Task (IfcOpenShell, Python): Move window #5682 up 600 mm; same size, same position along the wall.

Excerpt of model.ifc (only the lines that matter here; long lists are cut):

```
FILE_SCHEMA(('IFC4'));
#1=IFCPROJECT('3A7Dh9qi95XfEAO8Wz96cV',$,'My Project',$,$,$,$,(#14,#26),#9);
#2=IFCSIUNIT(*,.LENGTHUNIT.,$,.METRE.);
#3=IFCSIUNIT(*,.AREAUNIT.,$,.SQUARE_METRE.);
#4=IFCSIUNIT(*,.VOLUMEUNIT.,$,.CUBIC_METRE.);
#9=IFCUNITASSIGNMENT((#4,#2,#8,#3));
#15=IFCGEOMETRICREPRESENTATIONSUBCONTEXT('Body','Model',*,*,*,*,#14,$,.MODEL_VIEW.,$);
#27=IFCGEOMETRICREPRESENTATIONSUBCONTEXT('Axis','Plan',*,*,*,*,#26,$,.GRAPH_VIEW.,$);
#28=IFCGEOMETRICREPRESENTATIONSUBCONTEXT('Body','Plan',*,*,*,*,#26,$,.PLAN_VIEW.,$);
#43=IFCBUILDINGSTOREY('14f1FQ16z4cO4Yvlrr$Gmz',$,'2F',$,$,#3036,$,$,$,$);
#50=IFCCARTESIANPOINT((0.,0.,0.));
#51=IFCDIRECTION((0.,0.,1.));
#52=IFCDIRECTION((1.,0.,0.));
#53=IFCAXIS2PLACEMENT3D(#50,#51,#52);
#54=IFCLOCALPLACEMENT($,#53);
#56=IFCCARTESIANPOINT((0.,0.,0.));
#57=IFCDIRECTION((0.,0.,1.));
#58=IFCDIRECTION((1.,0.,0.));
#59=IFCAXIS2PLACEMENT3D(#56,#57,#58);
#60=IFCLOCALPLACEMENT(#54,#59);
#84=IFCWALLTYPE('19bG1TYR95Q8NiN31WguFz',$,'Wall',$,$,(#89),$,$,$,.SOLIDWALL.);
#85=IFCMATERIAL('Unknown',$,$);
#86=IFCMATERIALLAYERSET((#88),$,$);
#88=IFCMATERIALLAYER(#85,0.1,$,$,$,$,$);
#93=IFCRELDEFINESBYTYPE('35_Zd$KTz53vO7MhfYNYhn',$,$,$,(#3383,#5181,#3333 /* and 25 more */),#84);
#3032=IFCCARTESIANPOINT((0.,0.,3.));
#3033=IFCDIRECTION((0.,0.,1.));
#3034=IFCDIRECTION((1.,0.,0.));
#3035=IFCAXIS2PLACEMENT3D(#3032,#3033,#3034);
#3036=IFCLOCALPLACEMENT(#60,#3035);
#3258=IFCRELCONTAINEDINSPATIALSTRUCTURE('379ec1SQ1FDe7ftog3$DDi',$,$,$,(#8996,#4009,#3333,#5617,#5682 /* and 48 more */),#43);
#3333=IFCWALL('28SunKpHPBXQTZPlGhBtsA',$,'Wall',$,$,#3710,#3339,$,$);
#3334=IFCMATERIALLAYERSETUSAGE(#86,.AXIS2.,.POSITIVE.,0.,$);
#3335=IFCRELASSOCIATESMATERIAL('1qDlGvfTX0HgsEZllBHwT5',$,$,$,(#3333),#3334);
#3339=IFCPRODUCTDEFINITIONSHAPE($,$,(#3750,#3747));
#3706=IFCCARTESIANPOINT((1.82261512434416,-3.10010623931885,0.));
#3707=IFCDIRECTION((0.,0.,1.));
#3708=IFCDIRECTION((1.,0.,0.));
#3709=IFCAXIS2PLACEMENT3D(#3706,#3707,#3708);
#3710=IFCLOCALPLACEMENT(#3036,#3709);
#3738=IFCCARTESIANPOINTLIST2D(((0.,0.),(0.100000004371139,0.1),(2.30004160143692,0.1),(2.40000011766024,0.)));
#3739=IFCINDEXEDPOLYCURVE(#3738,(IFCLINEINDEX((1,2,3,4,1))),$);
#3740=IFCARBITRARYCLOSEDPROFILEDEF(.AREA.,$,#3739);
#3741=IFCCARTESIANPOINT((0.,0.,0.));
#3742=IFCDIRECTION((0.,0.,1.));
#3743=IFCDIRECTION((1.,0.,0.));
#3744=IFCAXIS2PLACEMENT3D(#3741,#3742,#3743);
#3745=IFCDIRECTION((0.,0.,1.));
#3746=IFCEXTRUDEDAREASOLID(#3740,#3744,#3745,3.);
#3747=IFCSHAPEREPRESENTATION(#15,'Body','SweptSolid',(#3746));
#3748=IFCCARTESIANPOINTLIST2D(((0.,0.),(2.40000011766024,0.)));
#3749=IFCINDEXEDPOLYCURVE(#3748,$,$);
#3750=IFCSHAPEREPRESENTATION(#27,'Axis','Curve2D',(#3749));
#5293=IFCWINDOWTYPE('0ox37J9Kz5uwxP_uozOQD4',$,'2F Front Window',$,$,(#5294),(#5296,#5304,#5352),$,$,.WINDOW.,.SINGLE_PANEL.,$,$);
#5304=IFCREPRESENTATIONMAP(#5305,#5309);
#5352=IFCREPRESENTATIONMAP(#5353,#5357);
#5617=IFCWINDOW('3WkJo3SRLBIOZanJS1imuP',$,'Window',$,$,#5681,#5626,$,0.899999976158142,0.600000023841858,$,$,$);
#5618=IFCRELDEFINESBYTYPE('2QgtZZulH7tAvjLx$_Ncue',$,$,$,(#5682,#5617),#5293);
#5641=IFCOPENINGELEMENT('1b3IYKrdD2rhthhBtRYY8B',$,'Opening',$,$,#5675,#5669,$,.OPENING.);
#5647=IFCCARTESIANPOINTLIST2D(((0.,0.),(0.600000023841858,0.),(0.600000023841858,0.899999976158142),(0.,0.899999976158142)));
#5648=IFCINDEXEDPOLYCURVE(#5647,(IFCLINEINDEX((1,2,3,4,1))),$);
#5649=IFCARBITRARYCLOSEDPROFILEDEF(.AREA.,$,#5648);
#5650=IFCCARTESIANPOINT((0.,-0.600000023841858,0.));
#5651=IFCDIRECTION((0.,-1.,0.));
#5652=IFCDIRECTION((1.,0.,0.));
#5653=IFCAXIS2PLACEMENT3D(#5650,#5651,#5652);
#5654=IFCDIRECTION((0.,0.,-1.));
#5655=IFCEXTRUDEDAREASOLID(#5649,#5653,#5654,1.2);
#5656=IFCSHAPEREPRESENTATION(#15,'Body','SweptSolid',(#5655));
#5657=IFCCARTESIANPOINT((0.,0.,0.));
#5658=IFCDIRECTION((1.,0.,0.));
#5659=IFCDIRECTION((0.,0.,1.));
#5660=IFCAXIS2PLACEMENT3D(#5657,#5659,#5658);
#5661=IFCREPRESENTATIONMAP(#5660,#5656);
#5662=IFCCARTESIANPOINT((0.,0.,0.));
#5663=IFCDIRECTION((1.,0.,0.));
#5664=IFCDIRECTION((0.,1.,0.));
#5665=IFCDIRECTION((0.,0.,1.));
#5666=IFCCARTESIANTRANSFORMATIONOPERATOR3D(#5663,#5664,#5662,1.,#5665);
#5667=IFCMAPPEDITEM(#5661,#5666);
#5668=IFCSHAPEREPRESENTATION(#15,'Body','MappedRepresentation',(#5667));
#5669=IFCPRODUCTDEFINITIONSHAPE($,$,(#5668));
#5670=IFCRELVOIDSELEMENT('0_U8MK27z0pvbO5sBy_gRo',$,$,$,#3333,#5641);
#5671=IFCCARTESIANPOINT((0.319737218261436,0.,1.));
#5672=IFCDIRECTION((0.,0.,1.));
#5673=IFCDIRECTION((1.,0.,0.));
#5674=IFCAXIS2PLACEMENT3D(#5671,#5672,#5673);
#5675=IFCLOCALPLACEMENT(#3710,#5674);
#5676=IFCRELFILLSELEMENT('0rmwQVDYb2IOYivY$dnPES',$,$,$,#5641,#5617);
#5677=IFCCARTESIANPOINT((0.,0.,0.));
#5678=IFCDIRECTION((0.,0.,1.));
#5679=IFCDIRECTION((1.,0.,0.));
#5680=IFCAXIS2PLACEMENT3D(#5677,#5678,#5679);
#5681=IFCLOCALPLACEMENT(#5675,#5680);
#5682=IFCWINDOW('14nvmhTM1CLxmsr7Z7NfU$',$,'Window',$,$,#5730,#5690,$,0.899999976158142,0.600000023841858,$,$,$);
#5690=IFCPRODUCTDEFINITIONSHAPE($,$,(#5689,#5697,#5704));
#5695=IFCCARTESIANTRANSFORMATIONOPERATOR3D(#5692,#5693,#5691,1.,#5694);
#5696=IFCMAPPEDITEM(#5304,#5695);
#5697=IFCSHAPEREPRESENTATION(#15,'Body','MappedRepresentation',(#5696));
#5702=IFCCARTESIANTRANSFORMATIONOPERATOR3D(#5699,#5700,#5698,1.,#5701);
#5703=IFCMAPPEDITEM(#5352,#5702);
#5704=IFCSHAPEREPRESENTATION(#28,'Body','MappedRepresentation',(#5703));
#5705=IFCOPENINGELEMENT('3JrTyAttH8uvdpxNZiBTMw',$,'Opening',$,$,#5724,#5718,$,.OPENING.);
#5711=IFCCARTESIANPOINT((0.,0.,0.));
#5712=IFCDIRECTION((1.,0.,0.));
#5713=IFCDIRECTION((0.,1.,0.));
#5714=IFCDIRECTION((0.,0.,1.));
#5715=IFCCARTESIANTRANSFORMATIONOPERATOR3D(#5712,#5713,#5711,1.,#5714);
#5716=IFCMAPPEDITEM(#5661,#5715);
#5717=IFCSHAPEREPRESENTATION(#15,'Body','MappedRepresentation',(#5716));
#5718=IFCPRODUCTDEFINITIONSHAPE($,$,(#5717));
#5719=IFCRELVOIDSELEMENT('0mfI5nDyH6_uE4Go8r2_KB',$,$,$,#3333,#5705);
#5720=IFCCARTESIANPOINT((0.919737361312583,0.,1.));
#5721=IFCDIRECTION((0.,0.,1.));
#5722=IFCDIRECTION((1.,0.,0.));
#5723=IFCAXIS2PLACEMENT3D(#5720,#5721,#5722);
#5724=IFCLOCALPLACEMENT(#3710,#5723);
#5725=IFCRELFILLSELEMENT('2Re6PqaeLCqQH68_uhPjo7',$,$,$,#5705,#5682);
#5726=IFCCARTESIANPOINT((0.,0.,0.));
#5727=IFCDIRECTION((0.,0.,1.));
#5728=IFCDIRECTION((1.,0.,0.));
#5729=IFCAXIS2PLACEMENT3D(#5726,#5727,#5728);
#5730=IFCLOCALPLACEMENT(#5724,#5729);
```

```python
import numpy as np
import ifcopenshell
import ifcopenshell.api.geometry
import ifcopenshell.util.placement
import ifcopenshell.util.unit

model = ifcopenshell.open("model.ifc")
unit_scale = ifcopenshell.util.unit.calculate_unit_scale(model)

window = model.by_guid("14nvmhTM1CLxmsr7Z7NfU$")
opening = window.FillsVoids[0].RelatingOpeningElement
dz = 0.6 / unit_scale

shift = np.array([0.0, 0.0, dz])
# The window is placed relative to its opening, so it follows when the opening moves.
matrix = ifcopenshell.util.placement.get_local_placement(opening.ObjectPlacement)
matrix[:3, 3] += shift
ifcopenshell.api.geometry.edit_object_placement(
    model, product=opening, matrix=matrix, is_si=False, should_transform_children=True
)

print(f"moved by {dz * unit_scale:+.3f} m")

model.write("model_rev.ifc")
```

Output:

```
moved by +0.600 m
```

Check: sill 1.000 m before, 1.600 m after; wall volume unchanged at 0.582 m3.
